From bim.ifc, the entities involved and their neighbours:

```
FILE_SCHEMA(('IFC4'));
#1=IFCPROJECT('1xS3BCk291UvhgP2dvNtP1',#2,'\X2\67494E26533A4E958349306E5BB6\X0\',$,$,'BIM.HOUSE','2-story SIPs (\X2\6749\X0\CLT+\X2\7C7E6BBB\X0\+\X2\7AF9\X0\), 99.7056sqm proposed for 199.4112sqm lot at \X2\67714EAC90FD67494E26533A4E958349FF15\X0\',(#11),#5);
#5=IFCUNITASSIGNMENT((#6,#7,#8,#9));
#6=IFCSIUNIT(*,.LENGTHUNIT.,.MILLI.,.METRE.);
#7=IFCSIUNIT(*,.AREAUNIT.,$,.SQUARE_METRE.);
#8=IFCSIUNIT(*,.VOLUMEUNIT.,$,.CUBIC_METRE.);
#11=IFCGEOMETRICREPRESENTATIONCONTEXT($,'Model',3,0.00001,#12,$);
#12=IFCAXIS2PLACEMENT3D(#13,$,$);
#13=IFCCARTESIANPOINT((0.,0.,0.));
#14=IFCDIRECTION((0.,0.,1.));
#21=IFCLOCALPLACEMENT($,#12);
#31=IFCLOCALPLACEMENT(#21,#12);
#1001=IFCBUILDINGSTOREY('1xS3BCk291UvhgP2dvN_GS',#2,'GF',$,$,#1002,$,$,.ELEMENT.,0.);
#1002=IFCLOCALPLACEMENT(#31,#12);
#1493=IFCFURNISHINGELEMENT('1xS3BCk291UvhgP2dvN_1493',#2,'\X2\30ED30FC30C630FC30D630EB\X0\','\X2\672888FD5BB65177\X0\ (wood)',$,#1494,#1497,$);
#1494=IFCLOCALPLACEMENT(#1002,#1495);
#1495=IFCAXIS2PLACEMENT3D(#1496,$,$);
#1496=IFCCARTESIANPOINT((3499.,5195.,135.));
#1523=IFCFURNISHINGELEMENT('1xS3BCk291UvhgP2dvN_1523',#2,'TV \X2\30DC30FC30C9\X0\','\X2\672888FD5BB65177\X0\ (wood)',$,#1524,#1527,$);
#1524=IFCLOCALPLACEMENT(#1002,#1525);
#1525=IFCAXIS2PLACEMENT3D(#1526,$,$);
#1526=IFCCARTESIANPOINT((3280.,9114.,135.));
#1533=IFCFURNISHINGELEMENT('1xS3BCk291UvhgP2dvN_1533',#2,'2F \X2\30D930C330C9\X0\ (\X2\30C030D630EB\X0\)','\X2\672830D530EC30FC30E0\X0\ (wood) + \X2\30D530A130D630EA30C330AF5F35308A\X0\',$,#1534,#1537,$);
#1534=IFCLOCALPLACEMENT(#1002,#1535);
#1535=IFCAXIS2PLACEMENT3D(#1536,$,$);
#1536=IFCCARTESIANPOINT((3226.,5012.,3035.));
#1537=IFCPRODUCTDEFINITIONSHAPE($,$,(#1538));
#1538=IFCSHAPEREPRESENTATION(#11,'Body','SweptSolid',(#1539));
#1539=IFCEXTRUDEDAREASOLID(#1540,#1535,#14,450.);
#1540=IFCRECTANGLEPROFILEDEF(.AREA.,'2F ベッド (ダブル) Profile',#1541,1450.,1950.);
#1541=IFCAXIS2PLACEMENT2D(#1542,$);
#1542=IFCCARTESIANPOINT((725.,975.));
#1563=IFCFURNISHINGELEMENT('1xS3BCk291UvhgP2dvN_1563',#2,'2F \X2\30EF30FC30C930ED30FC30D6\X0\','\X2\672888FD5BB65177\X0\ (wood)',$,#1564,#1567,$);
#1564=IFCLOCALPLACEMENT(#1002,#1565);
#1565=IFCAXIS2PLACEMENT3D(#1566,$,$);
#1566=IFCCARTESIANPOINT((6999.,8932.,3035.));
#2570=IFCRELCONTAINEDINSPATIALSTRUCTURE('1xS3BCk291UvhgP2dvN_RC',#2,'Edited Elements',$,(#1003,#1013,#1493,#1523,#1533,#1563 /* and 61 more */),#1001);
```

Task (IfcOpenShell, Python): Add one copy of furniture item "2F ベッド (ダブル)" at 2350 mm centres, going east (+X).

```python
import numpy as np
import ifcopenshell
import ifcopenshell.api.geometry
import ifcopenshell.api.root
import ifcopenshell.util.element
import ifcopenshell.util.placement
import ifcopenshell.util.unit

model = ifcopenshell.open("bim.ifc")
unit_scale = ifcopenshell.util.unit.calculate_unit_scale(model)


def reuse_history(source, copy):
    """copy_class also copies each property set's owner history, people and application; keep the originals."""
    for rel in copy.IsDefinedBy:
        if rel.is_a("IfcRelDefinesByProperties") and (history := rel.RelatingPropertyDefinition.OwnerHistory):
            rel.RelatingPropertyDefinition.OwnerHistory = source.OwnerHistory
            ifcopenshell.util.element.remove_deep2(model, history)


source = model.by_guid("1xS3BCk291UvhgP2dvN_1533")
base = ifcopenshell.util.placement.get_local_placement(source.ObjectPlacement)
step = np.array([1.0, 0.0, 0.0]) * 2.35 / unit_scale

for i in range(1, 2):
    copy = ifcopenshell.api.root.copy_class(model, product=source)
    copy.Representation = ifcopenshell.util.element.copy_deep(
        model, source.Representation, exclude=["IfcGeometricRepresentationContext", "IfcRepresentationMap"]
    )
    reuse_history(source, copy)
    matrix = base.copy()
    matrix[:3, 3] += i * step
    print("added at", matrix[:3, 3].round(3) + 0.0)
    ifcopenshell.api.geometry.edit_object_placement(model, product=copy, matrix=matrix, is_si=False)

model.write("bim_edited.ifc")
```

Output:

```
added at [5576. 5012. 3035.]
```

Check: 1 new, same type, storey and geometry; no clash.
